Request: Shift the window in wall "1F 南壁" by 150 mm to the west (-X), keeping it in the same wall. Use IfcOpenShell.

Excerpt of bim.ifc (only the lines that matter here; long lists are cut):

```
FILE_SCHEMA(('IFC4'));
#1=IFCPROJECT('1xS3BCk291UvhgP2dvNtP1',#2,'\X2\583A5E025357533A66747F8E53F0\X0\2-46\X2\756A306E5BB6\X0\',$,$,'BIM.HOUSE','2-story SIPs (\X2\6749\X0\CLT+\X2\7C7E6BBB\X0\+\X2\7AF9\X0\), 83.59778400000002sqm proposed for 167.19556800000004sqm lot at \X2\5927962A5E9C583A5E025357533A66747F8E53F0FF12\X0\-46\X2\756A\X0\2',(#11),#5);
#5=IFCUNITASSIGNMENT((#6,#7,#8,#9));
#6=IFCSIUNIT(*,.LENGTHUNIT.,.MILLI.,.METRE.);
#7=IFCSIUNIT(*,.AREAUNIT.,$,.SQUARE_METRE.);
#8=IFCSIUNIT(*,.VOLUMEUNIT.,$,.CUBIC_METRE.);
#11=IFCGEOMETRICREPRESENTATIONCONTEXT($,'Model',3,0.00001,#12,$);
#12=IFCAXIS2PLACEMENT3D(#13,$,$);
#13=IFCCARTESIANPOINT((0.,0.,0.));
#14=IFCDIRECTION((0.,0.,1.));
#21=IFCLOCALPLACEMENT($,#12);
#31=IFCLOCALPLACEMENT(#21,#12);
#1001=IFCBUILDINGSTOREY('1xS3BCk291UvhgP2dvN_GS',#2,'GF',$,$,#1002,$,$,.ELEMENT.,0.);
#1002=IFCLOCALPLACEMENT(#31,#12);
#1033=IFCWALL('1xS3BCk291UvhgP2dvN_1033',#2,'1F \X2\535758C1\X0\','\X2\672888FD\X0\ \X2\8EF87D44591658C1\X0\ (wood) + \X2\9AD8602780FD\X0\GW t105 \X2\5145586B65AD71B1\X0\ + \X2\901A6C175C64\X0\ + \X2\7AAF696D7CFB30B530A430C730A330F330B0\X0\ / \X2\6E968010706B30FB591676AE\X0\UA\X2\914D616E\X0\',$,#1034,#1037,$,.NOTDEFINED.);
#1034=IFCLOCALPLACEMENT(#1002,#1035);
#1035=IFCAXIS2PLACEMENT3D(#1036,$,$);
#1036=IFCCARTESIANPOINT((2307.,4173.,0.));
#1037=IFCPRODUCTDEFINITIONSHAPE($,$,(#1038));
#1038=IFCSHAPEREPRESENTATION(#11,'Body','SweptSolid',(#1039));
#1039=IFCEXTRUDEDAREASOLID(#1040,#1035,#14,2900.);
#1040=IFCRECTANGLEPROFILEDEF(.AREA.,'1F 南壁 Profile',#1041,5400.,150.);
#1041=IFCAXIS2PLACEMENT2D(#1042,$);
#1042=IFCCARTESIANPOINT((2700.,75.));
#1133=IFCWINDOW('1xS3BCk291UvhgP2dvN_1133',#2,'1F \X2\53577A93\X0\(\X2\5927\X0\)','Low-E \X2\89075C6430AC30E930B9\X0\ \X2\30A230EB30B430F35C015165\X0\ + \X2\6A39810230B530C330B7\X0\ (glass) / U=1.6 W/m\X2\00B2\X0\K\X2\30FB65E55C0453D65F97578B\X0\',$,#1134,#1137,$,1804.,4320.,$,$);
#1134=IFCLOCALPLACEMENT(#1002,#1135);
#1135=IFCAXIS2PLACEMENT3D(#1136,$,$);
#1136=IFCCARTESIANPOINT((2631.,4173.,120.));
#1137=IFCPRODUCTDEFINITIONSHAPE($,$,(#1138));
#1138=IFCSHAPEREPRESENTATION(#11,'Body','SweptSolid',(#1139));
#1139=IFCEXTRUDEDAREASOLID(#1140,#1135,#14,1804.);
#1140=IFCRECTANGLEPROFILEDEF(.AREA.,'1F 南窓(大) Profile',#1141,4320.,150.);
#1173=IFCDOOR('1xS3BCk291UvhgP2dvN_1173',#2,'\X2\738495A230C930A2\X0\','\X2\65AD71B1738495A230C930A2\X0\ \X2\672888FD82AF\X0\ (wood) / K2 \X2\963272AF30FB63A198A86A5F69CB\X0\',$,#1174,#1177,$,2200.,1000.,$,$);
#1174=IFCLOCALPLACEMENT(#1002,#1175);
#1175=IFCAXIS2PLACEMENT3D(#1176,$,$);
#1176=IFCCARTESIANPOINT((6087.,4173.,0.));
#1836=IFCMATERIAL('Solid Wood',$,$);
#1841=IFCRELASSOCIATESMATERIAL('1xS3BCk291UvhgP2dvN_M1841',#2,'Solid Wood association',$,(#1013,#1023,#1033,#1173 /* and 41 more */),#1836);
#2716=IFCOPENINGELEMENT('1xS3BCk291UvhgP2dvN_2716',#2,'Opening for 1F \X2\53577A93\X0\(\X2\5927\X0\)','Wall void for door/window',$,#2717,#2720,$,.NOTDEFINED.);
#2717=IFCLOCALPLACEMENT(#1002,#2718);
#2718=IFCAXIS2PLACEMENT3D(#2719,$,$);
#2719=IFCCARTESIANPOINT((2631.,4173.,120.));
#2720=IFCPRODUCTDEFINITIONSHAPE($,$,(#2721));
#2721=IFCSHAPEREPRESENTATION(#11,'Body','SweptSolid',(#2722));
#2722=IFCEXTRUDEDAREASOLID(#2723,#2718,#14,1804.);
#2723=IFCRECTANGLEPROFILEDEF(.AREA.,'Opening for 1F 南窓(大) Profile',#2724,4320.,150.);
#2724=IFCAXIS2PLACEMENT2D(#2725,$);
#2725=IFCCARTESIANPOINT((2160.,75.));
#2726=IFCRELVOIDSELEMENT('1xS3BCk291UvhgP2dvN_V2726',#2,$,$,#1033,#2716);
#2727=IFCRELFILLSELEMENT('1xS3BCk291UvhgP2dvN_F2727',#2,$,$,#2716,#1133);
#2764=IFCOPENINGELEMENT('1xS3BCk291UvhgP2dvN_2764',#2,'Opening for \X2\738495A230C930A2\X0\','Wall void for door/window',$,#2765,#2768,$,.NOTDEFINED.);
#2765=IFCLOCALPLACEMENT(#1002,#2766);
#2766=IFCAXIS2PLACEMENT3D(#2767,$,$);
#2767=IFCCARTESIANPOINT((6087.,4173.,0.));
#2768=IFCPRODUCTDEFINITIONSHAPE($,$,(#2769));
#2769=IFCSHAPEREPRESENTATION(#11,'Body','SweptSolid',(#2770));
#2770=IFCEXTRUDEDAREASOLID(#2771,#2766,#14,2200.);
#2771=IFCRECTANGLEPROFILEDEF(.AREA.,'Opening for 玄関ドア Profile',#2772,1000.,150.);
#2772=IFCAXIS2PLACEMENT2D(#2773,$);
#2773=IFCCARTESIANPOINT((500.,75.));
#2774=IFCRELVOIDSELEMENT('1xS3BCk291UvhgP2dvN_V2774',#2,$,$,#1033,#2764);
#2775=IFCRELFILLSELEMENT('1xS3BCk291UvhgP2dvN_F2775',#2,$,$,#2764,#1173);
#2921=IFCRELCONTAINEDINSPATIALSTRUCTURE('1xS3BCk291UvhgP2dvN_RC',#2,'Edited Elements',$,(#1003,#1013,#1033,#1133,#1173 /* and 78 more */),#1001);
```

```python
import ifcopenshell
import ifcopenshell.api.geometry
import ifcopenshell.util.placement
import ifcopenshell.util.unit

model = ifcopenshell.open("bim.ifc")
unit_scale = ifcopenshell.util.unit.calculate_unit_scale(model)

window = model.by_guid("1xS3BCk291UvhgP2dvN_1133")
opening = window.FillsVoids[0].RelatingOpeningElement
wall = opening.VoidsElements[0].RelatingBuildingElement

wall_matrix = ifcopenshell.util.placement.get_local_placement(wall.ObjectPlacement)
shift = wall_matrix[:3, 0] * -0.15 / unit_scale
before = ifcopenshell.util.placement.get_local_placement(window.ObjectPlacement)[:3, 3].copy()

# The window is not placed relative to its opening, so move both.
for product in (opening, window):
    matrix = ifcopenshell.util.placement.get_local_placement(product.ObjectPlacement)
    matrix[:3, 3] += shift
    ifcopenshell.api.geometry.edit_object_placement(model, product=product, matrix=matrix, is_si=False)

after = ifcopenshell.util.placement.get_local_placement(window.ObjectPlacement)[:3, 3]
print("window moved by", (after - before).round(3) + 0.0)

model.write("bim_v2.ifc")
```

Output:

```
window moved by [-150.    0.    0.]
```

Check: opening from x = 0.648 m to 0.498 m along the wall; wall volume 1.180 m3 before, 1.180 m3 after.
